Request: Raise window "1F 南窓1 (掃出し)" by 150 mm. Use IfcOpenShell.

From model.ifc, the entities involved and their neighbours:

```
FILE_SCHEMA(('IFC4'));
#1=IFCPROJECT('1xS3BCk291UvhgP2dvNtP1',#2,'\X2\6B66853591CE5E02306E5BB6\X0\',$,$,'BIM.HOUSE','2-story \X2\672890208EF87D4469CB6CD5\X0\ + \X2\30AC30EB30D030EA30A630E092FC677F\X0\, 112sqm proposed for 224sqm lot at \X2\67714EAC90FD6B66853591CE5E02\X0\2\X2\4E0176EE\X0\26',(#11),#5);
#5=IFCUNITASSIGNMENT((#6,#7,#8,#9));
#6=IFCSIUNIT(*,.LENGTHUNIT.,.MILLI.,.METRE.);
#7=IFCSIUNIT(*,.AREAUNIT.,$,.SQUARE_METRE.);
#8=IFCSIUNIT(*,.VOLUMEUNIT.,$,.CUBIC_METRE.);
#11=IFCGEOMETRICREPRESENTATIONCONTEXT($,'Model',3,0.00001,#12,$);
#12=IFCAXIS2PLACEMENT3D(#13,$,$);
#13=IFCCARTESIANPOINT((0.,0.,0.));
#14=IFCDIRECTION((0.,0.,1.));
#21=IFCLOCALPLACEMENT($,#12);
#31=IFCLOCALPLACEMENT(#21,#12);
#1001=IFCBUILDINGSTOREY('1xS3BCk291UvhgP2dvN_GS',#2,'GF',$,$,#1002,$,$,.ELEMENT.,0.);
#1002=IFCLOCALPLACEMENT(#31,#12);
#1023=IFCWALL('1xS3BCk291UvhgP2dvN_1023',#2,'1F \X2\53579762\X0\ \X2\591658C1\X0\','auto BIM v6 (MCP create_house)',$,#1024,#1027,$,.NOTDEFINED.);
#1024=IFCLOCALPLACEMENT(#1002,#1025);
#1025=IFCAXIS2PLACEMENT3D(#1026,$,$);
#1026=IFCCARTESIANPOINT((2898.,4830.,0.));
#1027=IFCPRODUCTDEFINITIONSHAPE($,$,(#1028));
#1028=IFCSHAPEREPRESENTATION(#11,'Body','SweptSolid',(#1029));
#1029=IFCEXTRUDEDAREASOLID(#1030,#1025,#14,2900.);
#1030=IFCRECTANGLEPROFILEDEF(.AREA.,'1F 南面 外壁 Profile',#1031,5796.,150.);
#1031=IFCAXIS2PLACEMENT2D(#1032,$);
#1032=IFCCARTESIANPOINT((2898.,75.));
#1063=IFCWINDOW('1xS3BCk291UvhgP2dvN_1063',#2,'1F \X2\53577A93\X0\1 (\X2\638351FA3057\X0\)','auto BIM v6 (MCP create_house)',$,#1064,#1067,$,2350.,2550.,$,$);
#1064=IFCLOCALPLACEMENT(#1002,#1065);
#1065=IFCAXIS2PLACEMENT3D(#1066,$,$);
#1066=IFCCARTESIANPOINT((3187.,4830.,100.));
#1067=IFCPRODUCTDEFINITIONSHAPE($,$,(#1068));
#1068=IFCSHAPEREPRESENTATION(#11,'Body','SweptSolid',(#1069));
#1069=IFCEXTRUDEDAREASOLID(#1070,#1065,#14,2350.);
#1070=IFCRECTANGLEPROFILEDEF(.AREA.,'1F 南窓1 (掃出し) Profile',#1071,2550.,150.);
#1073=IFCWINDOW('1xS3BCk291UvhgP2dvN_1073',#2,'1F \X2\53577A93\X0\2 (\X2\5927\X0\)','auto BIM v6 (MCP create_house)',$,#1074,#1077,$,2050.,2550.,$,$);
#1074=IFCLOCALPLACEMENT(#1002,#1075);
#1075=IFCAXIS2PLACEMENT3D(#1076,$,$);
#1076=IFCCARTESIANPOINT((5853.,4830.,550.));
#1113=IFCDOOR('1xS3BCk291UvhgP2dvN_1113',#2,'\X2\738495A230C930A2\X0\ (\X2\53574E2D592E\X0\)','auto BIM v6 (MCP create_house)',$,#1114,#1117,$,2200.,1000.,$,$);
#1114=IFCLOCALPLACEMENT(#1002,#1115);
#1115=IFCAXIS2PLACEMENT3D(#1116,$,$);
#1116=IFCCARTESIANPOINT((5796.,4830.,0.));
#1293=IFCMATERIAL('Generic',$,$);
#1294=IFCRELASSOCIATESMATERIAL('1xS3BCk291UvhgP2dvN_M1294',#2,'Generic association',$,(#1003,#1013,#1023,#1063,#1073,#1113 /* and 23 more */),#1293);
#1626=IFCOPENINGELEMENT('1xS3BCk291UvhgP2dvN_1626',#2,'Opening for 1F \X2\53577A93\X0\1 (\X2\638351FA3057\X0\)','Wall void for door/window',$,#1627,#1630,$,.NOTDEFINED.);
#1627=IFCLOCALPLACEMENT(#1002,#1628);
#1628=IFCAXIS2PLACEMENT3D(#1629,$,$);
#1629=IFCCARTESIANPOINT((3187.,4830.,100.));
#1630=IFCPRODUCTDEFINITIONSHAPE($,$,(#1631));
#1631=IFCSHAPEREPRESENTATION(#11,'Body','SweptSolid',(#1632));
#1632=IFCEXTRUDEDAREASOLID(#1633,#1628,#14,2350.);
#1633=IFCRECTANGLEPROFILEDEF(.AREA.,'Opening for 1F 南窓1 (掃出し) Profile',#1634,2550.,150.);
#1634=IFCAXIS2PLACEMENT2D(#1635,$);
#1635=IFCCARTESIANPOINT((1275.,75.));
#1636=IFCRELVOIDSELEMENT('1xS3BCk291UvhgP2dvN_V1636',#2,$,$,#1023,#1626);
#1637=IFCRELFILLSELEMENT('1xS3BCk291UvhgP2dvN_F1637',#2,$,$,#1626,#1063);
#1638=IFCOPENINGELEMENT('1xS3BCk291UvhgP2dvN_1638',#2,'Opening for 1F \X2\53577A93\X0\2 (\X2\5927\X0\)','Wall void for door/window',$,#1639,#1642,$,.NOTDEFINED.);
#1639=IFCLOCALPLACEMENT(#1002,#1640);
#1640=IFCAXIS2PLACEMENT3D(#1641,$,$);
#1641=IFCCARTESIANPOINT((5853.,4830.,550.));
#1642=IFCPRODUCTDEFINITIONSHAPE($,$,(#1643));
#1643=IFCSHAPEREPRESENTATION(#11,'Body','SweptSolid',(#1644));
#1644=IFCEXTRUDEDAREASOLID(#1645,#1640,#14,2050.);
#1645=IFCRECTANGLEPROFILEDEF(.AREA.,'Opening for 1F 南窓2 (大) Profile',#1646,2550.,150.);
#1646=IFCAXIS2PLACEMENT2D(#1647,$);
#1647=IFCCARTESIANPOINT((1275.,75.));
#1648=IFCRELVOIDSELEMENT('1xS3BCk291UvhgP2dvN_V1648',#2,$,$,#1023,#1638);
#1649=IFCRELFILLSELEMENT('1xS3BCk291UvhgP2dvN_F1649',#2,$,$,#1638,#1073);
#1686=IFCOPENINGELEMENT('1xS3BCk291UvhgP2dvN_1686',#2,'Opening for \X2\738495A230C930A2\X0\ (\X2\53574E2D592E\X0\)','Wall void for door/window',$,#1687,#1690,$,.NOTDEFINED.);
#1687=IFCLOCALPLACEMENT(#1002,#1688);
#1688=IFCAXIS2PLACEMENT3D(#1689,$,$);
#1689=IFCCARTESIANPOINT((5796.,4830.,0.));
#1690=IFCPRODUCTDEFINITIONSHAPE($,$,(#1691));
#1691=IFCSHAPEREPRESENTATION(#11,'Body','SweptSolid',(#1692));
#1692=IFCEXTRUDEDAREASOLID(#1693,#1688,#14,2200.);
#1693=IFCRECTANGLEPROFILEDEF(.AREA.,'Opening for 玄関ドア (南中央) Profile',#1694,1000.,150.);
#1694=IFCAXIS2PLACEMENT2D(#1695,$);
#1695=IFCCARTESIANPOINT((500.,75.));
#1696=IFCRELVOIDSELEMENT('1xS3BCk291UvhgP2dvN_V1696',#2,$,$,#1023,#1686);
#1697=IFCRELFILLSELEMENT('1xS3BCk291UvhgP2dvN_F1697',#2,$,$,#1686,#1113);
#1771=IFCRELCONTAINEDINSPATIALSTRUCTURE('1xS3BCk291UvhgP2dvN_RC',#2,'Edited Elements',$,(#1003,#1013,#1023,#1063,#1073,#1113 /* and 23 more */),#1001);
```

```python
import numpy as np
import ifcopenshell
import ifcopenshell.api.geometry
import ifcopenshell.util.placement
import ifcopenshell.util.unit

model = ifcopenshell.open("model.ifc")
unit_scale = ifcopenshell.util.unit.calculate_unit_scale(model)

window = model.by_guid("1xS3BCk291UvhgP2dvN_1063")
opening = window.FillsVoids[0].RelatingOpeningElement
dz = 0.15 / unit_scale

shift = np.array([0.0, 0.0, dz])
# The window is not placed relative to its opening, so move both.
for product in (opening, window):
    matrix = ifcopenshell.util.placement.get_local_placement(product.ObjectPlacement)
    matrix[:3, 3] += shift
    ifcopenshell.api.geometry.edit_object_placement(model, product=product, matrix=matrix, is_si=False)

print(f"moved by {dz * unit_scale:+.3f} m")

model.write("model-out.ifc")
```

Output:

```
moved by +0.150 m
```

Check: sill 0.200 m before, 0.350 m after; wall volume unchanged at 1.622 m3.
